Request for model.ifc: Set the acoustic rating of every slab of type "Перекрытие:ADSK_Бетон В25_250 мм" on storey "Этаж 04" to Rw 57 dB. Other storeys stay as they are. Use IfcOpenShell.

First a look at what the model holds.

```python
import ifcopenshell
import ifcopenshell.util.element

model = ifcopenshell.open("model.ifc")
print(model.schema)
storey = next(s for s in model.by_type("IfcBuildingStorey") if s.Name == "Этаж 04")
slabs = [e for e in ifcopenshell.util.element.get_decomposition(storey) if e.is_a("IfcSlab")]
seen = {}
for e in slabs:
    element_type = ifcopenshell.util.element.get_type(e)
    key = (element_type.Name if element_type != e and element_type else None, ifcopenshell.util.element.get_pset(e, "Pset_SlabCommon", "AcousticRating"))
    seen[key] = seen.get(key, 0) + 1
for (name, value), count in sorted(seen.items(), key=str):
    print(count, "x", name, "|", value)
```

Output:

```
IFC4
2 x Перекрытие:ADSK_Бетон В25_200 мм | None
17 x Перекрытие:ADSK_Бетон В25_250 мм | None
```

```python
import ifcopenshell
import ifcopenshell.api.pset
import ifcopenshell.util.element

model = ifcopenshell.open("model.ifc")

storey = next(s for s in model.by_type("IfcBuildingStorey") if s.Name == "Этаж 04")
slabs = [e for e in ifcopenshell.util.element.get_decomposition(storey) if e.is_a("IfcSlab")]

count = 0
for e in slabs:
    element_type = ifcopenshell.util.element.get_type(e)
    if element_type in (None, e) or element_type.Name != "Перекрытие:ADSK_Бетон В25_250 мм":
        continue
    # add_pset returns the element's existing set when there is one.
    pset = ifcopenshell.api.pset.add_pset(model, product=e, name="Pset_SlabCommon")
    ifcopenshell.api.pset.edit_pset(model, pset=pset, properties={"AcousticRating": "Rw 57 dB"})
    count += 1

print(count, "slabs updated")

model.write("model_v2.ifc")
```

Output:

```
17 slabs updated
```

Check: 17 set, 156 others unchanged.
